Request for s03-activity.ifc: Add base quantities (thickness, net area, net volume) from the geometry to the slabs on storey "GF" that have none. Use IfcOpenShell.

First a look at what the model holds.

```python
import ifcopenshell
import ifcopenshell.util.element
import ifcopenshell.util.unit

model = ifcopenshell.open("s03-activity.ifc")
print(model.schema)
for unit_type in ("LENGTHUNIT", "AREAUNIT", "VOLUMEUNIT"):
    print(unit_type, ifcopenshell.util.unit.calculate_unit_scale(model, unit_type))
storey = next(s for s in model.by_type("IfcBuildingStorey") if s.Name == "GF")
slabs = [e for e in ifcopenshell.util.element.get_decomposition(storey) if e.is_a("IfcSlab")]
for e in sorted(slabs, key=lambda e: e.id()):
    print(e.id(), e.is_a(), e.Name, list(ifcopenshell.util.element.get_psets(e, qtos_only=True)), sep=" | ")
```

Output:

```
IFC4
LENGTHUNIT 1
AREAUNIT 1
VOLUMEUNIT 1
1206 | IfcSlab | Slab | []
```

```python
import ifcopenshell
import ifcopenshell.api.pset
import ifcopenshell.geom
import ifcopenshell.util.element
import ifcopenshell.util.shape
import ifcopenshell.util.unit

model = ifcopenshell.open("s03-activity.ifc")
unit_scale = ifcopenshell.util.unit.calculate_unit_scale(model)
area_scale = ifcopenshell.util.unit.calculate_unit_scale(model, "AREAUNIT")
volume_scale = ifcopenshell.util.unit.calculate_unit_scale(model, "VOLUMEUNIT")
settings = ifcopenshell.geom.settings()

storey = next(s for s in model.by_type("IfcBuildingStorey") if s.Name == "GF")
slabs = [e for e in ifcopenshell.util.element.get_decomposition(storey) if e.is_a("IfcSlab")]

for e in sorted(slabs, key=lambda e: e.id()):
    if ifcopenshell.util.element.get_psets(e, qtos_only=True, should_inherit=False):
        continue
    # Geometry comes back in metres, in the element's own axes.
    shape = ifcopenshell.geom.create_shape(settings, e)
    values = {
        "Width": ifcopenshell.util.shape.get_z(shape.geometry) / unit_scale,
        "NetArea": ifcopenshell.util.shape.get_footprint_area(shape.geometry) / area_scale,
        "NetVolume": ifcopenshell.util.shape.get_volume(shape.geometry) / volume_scale,
    }
    qto = ifcopenshell.api.pset.add_qto(model, product=e, name="Qto_SlabBaseQuantities")
    ifcopenshell.api.pset.edit_qto(model, qto=qto, properties=values)
    print(e.id(), {k: round(v, 3) for k, v in values.items()})

model.write("s03-activity_edited.ifc")
```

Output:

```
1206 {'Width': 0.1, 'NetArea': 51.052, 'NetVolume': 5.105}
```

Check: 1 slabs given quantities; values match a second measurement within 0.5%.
